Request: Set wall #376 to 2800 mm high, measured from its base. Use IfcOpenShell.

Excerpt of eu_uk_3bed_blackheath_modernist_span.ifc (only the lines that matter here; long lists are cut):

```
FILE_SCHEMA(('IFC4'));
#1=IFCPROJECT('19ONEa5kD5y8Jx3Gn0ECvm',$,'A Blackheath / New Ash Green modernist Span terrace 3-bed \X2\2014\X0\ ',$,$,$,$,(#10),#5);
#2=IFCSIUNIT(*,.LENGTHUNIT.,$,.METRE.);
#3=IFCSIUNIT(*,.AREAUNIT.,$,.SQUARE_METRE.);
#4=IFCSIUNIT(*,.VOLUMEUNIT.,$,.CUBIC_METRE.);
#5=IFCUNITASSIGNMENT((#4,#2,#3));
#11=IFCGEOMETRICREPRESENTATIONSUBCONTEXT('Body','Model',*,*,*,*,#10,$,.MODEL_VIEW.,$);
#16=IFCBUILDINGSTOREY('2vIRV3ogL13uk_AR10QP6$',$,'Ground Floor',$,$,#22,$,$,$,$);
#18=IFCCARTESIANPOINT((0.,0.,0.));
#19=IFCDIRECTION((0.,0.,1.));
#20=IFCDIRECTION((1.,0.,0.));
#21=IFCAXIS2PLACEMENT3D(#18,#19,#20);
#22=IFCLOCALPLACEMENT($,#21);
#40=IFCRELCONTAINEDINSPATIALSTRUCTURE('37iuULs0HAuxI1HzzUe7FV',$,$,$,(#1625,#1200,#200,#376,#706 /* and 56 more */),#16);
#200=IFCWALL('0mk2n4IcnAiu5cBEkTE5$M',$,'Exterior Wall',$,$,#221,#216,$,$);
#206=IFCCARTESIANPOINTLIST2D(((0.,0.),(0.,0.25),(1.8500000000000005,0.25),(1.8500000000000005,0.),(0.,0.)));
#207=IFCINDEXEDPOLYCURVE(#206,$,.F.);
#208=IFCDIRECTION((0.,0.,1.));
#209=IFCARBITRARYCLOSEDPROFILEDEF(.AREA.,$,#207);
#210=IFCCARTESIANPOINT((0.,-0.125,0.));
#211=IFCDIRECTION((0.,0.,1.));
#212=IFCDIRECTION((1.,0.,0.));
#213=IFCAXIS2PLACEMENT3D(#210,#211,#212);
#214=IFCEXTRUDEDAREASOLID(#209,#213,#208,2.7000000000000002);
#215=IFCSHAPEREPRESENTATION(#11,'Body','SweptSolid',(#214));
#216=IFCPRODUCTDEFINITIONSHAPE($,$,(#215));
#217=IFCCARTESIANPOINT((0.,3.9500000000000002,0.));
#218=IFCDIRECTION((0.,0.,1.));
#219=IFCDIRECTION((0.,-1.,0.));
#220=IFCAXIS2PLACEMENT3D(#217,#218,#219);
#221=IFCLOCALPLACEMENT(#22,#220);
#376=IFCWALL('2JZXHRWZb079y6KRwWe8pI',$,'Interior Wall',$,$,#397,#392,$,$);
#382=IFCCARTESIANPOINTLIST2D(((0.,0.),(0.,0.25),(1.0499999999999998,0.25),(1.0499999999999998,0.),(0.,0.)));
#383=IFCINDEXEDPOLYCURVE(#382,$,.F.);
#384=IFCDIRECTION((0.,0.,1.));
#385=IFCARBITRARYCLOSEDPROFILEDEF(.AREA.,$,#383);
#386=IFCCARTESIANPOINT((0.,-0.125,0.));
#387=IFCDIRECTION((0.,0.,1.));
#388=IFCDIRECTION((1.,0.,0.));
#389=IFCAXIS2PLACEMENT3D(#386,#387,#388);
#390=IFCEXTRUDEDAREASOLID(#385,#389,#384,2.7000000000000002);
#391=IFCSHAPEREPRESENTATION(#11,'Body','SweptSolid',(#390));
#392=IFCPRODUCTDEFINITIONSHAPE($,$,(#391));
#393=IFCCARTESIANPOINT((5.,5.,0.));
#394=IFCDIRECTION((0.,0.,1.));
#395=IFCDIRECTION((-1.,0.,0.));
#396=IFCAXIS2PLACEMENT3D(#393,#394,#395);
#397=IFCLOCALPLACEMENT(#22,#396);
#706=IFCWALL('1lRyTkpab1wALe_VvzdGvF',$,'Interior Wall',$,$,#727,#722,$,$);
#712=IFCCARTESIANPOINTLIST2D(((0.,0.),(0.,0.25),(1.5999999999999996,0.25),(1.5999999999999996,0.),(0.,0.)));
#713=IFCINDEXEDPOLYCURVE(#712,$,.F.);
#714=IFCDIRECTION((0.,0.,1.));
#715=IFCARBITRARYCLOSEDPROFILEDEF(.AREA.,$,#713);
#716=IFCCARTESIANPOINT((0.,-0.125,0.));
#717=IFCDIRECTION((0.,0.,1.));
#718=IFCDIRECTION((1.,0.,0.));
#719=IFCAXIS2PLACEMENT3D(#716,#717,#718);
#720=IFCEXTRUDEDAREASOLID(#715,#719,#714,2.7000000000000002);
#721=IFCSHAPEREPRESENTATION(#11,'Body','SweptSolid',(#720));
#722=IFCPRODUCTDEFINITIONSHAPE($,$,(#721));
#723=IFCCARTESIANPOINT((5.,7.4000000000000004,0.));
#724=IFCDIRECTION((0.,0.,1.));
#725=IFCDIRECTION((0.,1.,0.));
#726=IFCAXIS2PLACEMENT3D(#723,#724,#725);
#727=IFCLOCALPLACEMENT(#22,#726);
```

```python
import ifcopenshell
import ifcopenshell.geom
import ifcopenshell.util.representation
import ifcopenshell.util.shape
import ifcopenshell.util.unit

model = ifcopenshell.open("eu_uk_3bed_blackheath_modernist_span.ifc")
unit_scale = ifcopenshell.util.unit.calculate_unit_scale(model)
settings = ifcopenshell.geom.settings()


def volume(element):
    """Net volume in cubic metres, openings subtracted."""
    shape = ifcopenshell.geom.create_shape(settings, element)
    return ifcopenshell.util.shape.get_volume(shape.geometry)


wall = model.by_guid("2JZXHRWZb079y6KRwWe8pI")
before = volume(wall)

body = ifcopenshell.util.representation.get_representation(wall, "Model", "Body")
solid = body.Items[0]
old_height = solid.Depth
solid.Depth = 2.8 / unit_scale
after = volume(wall)

print(f"height {old_height:g} -> {solid.Depth:g}, volume {before:.3f} -> {after:.3f} m3")

model.write("eu_uk_3bed_blackheath_modernist_span_edited.ifc")
```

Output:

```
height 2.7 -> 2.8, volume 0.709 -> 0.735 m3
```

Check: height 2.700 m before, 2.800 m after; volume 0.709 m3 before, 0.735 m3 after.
